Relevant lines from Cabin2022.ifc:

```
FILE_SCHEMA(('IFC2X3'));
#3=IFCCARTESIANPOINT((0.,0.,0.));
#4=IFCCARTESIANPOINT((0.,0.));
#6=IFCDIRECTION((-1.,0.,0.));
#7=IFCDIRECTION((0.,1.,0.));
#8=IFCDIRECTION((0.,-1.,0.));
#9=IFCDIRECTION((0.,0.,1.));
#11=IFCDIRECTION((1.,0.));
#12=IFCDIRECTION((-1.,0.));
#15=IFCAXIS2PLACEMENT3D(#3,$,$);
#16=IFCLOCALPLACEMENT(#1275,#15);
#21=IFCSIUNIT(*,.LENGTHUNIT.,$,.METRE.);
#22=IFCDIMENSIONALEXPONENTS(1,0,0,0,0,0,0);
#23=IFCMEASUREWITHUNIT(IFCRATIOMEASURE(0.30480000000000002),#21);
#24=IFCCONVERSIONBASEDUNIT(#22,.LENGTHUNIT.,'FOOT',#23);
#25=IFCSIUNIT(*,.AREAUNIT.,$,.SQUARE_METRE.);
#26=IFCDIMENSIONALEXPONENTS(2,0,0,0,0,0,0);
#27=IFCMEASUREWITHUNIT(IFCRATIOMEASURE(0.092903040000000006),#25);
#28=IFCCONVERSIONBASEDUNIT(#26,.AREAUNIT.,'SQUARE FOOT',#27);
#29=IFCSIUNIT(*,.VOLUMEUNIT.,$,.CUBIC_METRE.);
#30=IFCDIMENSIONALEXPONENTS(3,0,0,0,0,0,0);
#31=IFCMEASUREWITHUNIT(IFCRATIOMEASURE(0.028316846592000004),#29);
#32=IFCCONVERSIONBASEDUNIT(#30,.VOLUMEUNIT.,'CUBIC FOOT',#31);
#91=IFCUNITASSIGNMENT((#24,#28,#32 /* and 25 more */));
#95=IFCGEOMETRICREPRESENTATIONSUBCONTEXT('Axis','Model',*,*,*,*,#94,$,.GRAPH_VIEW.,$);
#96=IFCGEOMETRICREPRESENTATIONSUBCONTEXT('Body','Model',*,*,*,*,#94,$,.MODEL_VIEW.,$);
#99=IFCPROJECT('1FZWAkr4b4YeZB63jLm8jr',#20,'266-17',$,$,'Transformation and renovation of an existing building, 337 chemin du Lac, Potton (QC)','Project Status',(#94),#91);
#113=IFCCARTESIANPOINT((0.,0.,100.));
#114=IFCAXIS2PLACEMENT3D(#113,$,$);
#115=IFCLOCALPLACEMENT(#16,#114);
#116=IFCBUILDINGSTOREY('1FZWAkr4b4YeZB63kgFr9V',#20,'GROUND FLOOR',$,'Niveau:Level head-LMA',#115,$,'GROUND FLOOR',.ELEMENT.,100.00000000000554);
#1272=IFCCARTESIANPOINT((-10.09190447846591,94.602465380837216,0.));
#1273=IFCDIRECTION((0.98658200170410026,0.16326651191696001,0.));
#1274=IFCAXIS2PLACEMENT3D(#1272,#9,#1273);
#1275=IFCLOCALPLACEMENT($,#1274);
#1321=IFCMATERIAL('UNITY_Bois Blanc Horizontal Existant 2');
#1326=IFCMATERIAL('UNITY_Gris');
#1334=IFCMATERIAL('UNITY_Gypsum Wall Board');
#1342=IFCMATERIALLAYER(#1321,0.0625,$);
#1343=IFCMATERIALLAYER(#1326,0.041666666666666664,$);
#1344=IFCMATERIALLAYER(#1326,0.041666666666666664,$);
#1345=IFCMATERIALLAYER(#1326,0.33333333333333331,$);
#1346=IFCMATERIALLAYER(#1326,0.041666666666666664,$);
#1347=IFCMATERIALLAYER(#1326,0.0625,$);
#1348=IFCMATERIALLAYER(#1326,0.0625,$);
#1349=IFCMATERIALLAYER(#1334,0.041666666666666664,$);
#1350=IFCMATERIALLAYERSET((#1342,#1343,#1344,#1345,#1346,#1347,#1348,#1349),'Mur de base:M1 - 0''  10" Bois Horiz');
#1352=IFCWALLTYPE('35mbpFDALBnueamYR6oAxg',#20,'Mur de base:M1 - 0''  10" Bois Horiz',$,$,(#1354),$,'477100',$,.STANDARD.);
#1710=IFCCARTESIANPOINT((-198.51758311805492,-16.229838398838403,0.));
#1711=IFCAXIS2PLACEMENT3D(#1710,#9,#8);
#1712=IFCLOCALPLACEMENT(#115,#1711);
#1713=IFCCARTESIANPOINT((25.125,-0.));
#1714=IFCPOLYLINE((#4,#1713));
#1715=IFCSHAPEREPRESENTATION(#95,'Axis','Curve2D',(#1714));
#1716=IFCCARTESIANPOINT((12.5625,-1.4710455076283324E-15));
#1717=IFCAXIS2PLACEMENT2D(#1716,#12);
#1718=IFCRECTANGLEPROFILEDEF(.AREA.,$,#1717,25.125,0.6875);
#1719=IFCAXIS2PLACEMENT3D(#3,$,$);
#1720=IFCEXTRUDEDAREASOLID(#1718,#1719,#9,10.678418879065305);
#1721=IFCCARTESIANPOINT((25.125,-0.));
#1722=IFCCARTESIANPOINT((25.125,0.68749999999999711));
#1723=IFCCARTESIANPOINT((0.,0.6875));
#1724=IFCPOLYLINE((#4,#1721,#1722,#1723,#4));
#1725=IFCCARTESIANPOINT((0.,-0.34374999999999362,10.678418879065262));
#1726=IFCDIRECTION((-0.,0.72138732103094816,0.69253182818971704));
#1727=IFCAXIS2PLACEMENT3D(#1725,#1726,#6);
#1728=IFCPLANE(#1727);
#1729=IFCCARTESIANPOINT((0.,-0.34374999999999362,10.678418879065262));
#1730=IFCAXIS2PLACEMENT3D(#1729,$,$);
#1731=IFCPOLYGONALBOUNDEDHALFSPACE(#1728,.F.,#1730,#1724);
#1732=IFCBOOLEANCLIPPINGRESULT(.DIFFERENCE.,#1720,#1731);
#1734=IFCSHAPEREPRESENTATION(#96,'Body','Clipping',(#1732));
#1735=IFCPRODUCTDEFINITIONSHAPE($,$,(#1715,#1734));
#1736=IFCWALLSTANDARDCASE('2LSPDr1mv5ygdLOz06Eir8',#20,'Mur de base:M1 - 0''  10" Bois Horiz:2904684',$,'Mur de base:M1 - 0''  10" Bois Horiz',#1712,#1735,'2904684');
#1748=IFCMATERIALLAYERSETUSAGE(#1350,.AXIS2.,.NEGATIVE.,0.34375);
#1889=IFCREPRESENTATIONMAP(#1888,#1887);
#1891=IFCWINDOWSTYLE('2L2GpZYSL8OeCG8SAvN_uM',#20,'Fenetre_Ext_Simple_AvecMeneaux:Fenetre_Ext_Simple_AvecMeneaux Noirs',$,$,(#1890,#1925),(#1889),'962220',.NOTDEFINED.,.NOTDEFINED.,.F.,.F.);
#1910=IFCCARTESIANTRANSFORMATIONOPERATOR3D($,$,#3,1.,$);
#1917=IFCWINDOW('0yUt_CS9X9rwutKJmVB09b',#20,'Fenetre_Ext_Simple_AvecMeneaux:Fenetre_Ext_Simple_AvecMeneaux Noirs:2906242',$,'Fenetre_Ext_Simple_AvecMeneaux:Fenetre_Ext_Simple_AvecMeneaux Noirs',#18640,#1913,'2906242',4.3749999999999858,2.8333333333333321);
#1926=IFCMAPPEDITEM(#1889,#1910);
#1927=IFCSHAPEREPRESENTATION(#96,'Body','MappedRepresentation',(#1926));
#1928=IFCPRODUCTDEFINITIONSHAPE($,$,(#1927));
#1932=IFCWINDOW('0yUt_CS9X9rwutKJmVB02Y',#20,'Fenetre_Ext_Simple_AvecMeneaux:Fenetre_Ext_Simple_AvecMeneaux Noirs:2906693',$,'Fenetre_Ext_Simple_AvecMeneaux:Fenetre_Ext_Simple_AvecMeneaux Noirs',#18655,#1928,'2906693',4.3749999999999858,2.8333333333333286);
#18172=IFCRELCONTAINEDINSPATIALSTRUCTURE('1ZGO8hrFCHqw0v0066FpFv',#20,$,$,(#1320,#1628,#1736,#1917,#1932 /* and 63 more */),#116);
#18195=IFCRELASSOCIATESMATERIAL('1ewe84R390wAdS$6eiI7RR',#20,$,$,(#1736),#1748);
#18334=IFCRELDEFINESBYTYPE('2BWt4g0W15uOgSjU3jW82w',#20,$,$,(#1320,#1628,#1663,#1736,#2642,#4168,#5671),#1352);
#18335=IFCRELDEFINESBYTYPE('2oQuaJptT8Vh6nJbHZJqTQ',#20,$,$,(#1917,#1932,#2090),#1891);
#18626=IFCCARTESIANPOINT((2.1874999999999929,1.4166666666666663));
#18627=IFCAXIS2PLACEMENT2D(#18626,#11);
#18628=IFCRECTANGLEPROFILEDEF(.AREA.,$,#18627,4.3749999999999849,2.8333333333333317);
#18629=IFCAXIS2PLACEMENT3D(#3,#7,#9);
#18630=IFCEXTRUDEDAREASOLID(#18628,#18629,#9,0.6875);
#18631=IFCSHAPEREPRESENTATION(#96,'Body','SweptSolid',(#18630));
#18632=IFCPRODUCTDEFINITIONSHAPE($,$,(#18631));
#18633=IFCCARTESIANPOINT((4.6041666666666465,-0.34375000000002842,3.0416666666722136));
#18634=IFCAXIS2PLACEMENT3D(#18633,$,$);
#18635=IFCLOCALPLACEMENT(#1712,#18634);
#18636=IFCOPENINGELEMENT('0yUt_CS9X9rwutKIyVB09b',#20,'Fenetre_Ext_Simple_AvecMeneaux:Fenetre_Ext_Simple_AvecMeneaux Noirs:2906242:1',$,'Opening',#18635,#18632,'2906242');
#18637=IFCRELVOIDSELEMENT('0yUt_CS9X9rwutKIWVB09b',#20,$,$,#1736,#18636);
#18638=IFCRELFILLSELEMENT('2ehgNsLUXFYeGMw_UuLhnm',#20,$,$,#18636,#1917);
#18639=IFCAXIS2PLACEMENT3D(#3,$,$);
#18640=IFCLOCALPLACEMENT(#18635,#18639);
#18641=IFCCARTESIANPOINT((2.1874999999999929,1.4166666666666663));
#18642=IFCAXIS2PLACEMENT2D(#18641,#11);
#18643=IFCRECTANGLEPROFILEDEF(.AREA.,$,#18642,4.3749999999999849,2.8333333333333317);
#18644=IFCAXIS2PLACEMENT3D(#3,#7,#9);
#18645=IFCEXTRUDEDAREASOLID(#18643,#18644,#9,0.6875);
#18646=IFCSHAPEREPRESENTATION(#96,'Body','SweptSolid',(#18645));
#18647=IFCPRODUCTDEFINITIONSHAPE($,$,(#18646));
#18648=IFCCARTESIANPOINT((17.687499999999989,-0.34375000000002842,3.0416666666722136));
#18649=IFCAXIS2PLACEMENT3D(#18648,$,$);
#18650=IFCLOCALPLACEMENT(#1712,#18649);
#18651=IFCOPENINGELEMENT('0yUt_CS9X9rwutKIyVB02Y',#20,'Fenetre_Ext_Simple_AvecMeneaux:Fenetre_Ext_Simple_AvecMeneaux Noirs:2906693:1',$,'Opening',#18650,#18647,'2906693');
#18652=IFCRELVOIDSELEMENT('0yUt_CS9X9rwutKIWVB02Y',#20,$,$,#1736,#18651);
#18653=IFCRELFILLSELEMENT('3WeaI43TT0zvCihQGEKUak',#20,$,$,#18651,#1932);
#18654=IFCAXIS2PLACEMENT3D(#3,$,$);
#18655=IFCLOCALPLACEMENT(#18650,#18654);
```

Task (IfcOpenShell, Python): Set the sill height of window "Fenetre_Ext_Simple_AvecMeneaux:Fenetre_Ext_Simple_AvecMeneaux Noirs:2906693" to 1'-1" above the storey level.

```python
import numpy as np
import ifcopenshell
import ifcopenshell.api.geometry
import ifcopenshell.geom
import ifcopenshell.util.element
import ifcopenshell.util.placement
import ifcopenshell.util.shape
import ifcopenshell.util.unit

model = ifcopenshell.open("Cabin2022.ifc")
unit_scale = ifcopenshell.util.unit.calculate_unit_scale(model)

window = model.by_guid("0yUt_CS9X9rwutKJmVB02Y")
opening = window.FillsVoids[0].RelatingOpeningElement
storey = ifcopenshell.util.element.get_container(window, ifc_class="IfcBuildingStorey")
level = ifcopenshell.util.placement.get_local_placement(storey.ObjectPlacement)[2, 3]

# The opening's origin need not be at the sill, so measure its lowest point.
shape = ifcopenshell.geom.create_shape(ifcopenshell.geom.settings(), opening)
bottom = ifcopenshell.util.shape.get_shape_bottom_elevation(shape, shape.geometry) / unit_scale
dz = level + 13 * 0.0254 / unit_scale - bottom

shift = np.array([0.0, 0.0, dz])
# The window is placed relative to its opening, so it follows when the opening moves.
matrix = ifcopenshell.util.placement.get_local_placement(opening.ObjectPlacement)
matrix[:3, 3] += shift
ifcopenshell.api.geometry.edit_object_placement(
    model, product=opening, matrix=matrix, is_si=False, should_transform_children=True
)

print(f"moved by {dz * unit_scale:+.3f} m")

model.write("Cabin2022_v2.ifc")
```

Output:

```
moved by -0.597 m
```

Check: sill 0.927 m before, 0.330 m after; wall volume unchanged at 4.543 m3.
